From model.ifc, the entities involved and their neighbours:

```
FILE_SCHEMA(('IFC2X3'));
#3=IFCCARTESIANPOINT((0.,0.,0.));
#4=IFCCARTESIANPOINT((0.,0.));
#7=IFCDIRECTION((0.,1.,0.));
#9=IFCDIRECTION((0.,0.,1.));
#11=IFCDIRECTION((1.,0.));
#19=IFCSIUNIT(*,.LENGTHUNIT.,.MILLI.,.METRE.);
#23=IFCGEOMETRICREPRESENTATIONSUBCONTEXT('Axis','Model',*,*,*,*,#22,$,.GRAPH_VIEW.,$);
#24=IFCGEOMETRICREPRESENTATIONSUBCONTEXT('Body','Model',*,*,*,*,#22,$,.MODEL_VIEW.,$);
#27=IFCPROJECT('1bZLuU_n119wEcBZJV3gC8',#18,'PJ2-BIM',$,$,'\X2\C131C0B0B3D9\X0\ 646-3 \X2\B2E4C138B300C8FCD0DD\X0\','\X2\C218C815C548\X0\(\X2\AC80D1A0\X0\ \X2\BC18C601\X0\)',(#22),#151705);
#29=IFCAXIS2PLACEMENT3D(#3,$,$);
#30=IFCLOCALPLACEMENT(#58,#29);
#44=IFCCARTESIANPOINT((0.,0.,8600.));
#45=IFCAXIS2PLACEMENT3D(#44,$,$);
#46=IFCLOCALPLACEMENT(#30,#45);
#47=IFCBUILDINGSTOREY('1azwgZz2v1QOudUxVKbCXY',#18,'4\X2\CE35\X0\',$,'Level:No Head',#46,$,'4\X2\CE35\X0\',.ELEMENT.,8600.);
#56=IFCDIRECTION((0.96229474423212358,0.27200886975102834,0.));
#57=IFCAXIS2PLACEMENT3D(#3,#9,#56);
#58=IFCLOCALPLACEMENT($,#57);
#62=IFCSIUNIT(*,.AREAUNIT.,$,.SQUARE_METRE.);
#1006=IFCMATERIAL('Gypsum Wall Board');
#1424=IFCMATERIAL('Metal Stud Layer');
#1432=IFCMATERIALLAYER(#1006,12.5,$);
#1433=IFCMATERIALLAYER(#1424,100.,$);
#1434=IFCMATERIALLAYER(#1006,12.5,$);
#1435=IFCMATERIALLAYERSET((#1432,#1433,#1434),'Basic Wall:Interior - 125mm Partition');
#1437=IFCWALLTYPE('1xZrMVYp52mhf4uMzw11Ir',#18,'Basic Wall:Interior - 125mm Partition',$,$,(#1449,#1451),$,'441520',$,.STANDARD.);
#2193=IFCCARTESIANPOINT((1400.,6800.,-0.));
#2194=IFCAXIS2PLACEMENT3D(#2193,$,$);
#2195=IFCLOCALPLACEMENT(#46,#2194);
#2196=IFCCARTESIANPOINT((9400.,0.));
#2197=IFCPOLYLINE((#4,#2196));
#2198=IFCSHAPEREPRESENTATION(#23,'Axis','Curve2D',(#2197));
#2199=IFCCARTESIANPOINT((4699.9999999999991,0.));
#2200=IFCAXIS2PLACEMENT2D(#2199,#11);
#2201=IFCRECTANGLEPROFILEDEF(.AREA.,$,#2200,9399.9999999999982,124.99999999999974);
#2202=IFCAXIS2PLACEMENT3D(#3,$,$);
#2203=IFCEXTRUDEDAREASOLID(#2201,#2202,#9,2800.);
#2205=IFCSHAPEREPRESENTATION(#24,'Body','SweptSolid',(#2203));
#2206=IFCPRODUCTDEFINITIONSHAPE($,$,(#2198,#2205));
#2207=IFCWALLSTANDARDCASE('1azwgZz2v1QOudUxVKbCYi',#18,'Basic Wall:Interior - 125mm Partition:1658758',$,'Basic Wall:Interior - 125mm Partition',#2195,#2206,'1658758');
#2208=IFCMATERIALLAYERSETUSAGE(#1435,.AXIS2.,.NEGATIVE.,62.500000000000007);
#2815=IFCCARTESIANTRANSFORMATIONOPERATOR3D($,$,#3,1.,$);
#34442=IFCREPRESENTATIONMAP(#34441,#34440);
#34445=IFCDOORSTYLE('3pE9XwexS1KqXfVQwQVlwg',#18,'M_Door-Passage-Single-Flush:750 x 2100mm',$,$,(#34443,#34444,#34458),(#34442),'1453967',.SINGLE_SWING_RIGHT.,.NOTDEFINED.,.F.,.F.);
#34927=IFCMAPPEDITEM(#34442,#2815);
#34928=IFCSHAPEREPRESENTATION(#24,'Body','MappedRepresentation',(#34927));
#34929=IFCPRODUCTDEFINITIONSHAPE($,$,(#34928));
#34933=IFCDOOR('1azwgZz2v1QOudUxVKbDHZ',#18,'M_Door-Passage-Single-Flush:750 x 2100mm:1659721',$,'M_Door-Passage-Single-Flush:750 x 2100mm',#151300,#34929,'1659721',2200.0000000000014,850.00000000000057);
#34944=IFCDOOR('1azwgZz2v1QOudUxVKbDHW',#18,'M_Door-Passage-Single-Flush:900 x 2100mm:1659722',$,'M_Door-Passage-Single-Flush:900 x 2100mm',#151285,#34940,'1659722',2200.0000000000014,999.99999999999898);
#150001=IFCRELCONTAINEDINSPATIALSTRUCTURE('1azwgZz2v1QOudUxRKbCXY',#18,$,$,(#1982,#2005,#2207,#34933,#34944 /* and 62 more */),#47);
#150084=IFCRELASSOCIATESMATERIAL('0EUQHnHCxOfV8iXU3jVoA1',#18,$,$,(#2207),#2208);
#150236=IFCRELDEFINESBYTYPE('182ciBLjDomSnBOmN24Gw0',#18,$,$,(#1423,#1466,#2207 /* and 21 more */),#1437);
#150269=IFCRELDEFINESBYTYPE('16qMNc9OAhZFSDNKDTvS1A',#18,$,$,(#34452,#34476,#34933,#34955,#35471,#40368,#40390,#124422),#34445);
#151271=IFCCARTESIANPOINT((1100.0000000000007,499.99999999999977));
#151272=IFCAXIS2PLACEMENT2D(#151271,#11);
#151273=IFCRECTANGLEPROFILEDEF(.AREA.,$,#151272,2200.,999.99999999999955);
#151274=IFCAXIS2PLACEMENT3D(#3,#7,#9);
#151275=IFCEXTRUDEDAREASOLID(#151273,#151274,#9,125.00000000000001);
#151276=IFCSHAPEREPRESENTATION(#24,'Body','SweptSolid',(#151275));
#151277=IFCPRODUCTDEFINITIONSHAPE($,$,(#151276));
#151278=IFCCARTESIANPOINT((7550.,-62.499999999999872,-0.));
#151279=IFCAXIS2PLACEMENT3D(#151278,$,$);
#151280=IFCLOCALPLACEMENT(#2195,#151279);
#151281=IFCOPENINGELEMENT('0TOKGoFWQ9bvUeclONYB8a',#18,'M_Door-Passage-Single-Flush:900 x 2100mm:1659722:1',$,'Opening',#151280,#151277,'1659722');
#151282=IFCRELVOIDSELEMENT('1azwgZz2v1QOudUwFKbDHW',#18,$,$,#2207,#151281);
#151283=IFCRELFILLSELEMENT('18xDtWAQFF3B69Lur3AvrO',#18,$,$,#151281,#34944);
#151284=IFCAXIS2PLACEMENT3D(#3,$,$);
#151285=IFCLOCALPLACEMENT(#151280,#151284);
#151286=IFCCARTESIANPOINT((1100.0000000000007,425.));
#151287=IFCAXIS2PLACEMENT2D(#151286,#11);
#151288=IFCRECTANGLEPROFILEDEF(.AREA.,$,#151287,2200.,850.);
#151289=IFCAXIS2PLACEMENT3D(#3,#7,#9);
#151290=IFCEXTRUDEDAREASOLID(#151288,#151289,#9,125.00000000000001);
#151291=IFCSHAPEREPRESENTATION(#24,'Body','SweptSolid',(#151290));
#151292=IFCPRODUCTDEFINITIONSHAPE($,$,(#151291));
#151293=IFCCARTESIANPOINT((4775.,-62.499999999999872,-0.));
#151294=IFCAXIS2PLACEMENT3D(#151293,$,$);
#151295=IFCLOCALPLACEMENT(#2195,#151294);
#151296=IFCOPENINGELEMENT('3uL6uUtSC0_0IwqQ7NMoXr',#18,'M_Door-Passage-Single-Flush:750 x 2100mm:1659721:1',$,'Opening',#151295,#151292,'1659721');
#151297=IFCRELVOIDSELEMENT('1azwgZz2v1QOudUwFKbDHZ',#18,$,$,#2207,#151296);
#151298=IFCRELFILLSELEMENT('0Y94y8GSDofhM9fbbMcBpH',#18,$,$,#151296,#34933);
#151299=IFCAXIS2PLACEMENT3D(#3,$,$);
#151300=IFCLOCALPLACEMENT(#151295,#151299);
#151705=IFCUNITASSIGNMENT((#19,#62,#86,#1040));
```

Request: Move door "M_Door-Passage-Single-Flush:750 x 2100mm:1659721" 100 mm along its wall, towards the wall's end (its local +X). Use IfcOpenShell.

```python
import ifcopenshell
import ifcopenshell.api.geometry
import ifcopenshell.util.placement

model = ifcopenshell.open("model.ifc")

door = model.by_guid("1azwgZz2v1QOudUxVKbDHZ")
opening = door.FillsVoids[0].RelatingOpeningElement
wall = opening.VoidsElements[0].RelatingBuildingElement

wall_matrix = ifcopenshell.util.placement.get_local_placement(wall.ObjectPlacement)
shift = wall_matrix[:3, 0] * 100.0
before = ifcopenshell.util.placement.get_local_placement(door.ObjectPlacement)[:3, 3].copy()

# The door is placed relative to its opening, so it follows when the opening moves.
matrix = ifcopenshell.util.placement.get_local_placement(opening.ObjectPlacement)
matrix[:3, 3] += shift
ifcopenshell.api.geometry.edit_object_placement(
    model, product=opening, matrix=matrix, is_si=False, should_transform_children=True
)

after = ifcopenshell.util.placement.get_local_placement(door.ObjectPlacement)[:3, 3]
print("door moved by", (after - before).round(3) + 0.0)

model.write("model-out.ifc")
```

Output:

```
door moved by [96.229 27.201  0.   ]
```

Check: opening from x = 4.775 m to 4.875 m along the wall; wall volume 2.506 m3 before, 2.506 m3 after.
